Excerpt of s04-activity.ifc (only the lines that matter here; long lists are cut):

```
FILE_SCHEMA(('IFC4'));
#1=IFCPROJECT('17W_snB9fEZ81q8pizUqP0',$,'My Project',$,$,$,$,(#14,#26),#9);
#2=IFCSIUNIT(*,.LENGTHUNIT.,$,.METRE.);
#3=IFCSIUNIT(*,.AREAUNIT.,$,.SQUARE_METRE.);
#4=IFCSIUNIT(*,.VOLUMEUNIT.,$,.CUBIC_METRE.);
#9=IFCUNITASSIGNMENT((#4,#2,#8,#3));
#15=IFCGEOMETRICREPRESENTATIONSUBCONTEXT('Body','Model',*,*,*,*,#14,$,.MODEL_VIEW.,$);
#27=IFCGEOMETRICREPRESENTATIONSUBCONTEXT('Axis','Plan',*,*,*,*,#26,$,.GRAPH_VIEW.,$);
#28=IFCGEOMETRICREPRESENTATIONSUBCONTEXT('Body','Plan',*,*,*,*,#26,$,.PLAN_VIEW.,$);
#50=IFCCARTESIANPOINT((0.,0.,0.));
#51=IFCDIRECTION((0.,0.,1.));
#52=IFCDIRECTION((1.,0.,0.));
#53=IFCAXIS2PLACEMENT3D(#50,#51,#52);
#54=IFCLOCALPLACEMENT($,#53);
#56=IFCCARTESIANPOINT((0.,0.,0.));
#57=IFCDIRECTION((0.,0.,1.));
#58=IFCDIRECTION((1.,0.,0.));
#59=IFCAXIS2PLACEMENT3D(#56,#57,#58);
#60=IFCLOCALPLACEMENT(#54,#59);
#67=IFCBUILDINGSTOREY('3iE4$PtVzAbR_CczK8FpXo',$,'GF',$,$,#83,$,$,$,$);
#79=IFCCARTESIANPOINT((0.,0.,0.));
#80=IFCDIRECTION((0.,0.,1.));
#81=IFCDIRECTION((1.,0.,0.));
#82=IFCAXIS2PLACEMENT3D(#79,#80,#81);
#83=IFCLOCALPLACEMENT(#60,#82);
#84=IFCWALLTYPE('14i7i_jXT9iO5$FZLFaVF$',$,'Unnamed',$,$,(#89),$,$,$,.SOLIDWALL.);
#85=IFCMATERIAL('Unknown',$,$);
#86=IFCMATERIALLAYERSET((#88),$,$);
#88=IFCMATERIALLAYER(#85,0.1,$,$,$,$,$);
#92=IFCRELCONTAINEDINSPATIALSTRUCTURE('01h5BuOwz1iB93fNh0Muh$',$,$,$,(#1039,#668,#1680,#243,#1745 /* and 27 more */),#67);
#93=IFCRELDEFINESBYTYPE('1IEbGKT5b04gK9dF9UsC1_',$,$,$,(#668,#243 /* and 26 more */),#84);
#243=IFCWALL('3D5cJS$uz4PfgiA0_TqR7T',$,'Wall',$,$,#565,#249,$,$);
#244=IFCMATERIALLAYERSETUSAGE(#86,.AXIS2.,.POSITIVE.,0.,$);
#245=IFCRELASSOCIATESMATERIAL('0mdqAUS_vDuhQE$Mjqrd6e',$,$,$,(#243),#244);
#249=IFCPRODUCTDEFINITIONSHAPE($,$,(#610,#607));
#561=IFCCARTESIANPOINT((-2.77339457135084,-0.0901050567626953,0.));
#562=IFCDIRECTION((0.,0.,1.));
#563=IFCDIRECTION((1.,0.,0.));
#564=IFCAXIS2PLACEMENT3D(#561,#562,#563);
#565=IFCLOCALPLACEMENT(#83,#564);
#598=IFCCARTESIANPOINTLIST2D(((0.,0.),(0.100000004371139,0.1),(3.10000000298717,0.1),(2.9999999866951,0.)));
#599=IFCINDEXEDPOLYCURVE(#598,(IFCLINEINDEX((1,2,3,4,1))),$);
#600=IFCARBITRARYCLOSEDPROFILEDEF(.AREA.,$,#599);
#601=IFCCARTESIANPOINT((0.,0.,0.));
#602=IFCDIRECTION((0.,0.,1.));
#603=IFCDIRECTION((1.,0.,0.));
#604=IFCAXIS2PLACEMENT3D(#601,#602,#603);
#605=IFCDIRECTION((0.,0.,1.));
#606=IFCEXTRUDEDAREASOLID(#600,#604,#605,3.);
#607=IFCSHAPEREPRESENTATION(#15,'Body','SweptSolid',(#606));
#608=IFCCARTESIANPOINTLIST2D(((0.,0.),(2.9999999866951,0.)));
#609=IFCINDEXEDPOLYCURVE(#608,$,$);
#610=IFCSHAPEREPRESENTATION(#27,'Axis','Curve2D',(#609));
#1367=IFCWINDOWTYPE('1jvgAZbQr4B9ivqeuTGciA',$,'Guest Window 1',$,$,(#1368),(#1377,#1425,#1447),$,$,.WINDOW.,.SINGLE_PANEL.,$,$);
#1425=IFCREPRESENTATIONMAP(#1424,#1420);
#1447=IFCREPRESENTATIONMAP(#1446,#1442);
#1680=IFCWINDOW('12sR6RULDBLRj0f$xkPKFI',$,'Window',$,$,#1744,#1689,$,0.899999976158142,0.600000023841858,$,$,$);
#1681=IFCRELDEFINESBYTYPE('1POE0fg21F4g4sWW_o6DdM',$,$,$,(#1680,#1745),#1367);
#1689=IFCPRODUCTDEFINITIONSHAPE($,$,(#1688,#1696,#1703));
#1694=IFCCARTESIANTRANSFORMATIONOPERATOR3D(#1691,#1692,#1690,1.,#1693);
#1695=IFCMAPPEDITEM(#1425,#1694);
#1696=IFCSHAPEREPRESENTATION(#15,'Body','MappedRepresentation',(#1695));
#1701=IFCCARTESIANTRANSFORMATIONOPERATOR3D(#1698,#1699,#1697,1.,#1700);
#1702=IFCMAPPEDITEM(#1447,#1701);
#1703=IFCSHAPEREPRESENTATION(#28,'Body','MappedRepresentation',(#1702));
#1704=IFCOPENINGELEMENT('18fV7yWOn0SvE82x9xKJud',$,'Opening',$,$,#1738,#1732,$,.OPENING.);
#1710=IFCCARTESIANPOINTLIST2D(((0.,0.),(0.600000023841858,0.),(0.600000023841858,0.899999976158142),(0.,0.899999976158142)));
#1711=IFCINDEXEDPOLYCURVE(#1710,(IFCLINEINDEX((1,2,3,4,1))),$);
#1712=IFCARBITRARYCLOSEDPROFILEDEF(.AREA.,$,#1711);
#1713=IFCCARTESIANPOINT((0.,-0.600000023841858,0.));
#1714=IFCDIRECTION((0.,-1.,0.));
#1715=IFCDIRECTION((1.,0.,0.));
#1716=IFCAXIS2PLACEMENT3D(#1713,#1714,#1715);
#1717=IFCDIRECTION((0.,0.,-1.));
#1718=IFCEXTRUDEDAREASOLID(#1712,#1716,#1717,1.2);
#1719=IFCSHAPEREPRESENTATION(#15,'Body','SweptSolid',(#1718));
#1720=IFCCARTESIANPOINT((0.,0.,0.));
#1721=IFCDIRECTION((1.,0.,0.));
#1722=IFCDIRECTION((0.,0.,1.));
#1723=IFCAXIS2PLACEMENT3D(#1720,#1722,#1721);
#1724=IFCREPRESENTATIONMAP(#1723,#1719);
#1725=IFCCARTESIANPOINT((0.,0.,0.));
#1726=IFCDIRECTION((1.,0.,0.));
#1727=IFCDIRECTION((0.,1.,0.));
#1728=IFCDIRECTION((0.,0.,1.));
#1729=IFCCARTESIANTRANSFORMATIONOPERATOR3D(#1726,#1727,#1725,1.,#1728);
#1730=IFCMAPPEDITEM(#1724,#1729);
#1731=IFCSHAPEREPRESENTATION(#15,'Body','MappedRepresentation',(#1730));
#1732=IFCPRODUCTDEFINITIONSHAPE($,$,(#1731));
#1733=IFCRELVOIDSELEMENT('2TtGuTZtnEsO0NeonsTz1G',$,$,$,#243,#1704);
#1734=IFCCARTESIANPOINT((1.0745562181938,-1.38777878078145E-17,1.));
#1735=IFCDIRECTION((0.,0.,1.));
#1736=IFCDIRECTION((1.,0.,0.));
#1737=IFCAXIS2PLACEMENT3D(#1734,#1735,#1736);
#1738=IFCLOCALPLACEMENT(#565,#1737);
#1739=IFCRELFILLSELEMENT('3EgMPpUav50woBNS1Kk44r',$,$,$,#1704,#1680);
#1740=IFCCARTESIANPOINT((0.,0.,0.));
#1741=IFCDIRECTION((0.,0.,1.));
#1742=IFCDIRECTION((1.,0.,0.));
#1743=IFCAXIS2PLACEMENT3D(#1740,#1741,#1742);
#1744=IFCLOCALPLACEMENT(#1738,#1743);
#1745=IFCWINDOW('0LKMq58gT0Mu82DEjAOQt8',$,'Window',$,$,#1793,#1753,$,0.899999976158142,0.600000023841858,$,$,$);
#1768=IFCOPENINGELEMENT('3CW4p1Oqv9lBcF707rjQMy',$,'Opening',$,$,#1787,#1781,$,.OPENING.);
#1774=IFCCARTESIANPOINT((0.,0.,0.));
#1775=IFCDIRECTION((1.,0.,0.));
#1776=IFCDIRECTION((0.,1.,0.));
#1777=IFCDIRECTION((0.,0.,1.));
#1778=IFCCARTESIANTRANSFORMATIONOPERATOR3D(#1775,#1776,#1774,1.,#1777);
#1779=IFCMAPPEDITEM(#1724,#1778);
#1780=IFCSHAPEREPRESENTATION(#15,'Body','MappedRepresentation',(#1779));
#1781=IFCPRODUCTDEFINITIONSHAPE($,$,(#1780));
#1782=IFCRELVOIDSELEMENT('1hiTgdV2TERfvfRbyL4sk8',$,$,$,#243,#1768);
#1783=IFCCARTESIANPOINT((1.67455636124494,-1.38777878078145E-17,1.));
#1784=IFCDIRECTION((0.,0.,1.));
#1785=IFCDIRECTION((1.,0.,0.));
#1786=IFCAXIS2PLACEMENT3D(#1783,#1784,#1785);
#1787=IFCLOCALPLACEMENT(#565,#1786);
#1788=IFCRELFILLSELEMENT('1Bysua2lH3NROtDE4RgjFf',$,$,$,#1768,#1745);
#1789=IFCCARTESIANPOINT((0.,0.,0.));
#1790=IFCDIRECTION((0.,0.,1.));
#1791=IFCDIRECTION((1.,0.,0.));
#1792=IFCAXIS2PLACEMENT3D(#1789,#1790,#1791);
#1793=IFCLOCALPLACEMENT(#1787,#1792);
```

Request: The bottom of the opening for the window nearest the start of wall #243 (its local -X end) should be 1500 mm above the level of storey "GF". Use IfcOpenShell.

```python
import numpy as np
import ifcopenshell
import ifcopenshell.api.geometry
import ifcopenshell.geom
import ifcopenshell.util.element
import ifcopenshell.util.placement
import ifcopenshell.util.shape
import ifcopenshell.util.unit

model = ifcopenshell.open("s04-activity.ifc")
unit_scale = ifcopenshell.util.unit.calculate_unit_scale(model)

window = model.by_guid("12sR6RULDBLRj0f$xkPKFI")
opening = window.FillsVoids[0].RelatingOpeningElement
storey = ifcopenshell.util.element.get_container(window, ifc_class="IfcBuildingStorey")
level = ifcopenshell.util.placement.get_local_placement(storey.ObjectPlacement)[2, 3]

# The opening's origin need not be at the sill, so measure its lowest point.
shape = ifcopenshell.geom.create_shape(ifcopenshell.geom.settings(), opening)
bottom = ifcopenshell.util.shape.get_shape_bottom_elevation(shape, shape.geometry) / unit_scale
dz = level + 1.5 - bottom

shift = np.array([0.0, 0.0, dz])
# The window is placed relative to its opening, so it follows when the opening moves.
matrix = ifcopenshell.util.placement.get_local_placement(opening.ObjectPlacement)
matrix[:3, 3] += shift
ifcopenshell.api.geometry.edit_object_placement(
    model, product=opening, matrix=matrix, is_si=False, should_transform_children=True
)

print(f"moved by {dz * unit_scale:+.3f} m")

model.write("s04-activity-out.ifc")
```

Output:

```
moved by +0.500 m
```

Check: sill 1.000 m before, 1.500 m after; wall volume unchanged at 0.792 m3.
